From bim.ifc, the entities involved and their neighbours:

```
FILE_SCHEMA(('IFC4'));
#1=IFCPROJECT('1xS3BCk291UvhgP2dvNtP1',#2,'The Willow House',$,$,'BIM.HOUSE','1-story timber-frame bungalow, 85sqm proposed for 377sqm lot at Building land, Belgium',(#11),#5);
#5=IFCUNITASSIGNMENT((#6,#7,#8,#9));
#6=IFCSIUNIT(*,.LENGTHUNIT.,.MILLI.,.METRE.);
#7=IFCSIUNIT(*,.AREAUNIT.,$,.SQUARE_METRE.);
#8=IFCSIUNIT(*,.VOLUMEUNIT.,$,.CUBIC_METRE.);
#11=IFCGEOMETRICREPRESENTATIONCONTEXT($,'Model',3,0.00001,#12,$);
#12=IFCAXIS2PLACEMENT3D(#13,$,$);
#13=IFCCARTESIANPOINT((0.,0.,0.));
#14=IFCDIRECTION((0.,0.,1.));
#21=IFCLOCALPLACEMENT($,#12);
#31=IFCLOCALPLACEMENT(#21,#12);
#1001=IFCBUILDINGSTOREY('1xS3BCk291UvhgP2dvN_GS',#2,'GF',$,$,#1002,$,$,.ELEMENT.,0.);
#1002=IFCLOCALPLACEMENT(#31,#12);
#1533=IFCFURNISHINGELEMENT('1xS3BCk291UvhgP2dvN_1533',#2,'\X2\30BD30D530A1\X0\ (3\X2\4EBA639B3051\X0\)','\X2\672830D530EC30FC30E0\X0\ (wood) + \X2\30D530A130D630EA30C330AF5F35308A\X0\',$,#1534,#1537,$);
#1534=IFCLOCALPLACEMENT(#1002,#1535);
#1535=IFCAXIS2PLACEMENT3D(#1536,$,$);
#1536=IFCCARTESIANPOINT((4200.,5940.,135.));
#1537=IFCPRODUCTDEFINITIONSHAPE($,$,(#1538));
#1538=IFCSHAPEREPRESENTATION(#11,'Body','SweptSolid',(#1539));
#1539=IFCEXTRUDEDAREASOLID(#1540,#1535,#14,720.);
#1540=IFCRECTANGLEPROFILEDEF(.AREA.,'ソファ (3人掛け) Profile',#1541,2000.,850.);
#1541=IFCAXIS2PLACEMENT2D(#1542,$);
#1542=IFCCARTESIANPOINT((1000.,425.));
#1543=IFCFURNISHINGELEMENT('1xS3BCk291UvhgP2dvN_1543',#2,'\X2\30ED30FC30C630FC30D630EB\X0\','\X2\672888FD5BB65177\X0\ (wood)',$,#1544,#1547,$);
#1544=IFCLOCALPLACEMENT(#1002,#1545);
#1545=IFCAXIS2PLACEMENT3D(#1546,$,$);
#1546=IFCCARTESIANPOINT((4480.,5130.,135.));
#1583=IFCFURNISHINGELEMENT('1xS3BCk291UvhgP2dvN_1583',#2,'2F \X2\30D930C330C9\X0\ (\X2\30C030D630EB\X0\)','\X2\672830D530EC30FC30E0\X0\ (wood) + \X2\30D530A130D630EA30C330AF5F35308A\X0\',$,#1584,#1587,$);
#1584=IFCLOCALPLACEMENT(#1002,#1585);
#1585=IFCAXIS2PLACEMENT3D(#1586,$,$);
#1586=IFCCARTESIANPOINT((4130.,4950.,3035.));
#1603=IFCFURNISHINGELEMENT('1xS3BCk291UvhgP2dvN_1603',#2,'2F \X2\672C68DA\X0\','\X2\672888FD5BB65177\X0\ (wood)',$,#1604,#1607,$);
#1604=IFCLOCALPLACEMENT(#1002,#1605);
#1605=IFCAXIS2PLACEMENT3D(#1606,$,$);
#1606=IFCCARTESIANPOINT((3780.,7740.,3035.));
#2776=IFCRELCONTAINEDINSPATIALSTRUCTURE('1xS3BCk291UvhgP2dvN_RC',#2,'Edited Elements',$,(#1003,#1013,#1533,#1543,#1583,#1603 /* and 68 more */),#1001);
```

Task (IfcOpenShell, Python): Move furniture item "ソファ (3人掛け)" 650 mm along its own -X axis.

```python
import ifcopenshell
import ifcopenshell.api.geometry
import ifcopenshell.util.placement
import ifcopenshell.util.unit

model = ifcopenshell.open("bim.ifc")
unit_scale = ifcopenshell.util.unit.calculate_unit_scale(model)

item = model.by_id(1533)
matrix = ifcopenshell.util.placement.get_local_placement(item.ObjectPlacement)
matrix[:3, 3] -= matrix[:3, 0] * 0.65 / unit_scale
ifcopenshell.api.geometry.edit_object_placement(model, product=item, matrix=matrix, is_si=False)

print(ifcopenshell.util.placement.get_local_placement(item.ObjectPlacement).round(3) + 0.0)

model.write("bim_rev.ifc")
```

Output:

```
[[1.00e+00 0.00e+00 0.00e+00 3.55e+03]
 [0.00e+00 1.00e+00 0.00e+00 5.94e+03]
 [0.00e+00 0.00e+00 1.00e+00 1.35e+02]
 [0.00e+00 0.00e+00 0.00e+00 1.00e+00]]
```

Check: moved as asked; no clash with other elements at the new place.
